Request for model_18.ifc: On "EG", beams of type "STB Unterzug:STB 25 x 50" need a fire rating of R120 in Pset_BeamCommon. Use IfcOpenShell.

First a look at what the model holds.

```python
import ifcopenshell
import ifcopenshell.util.element

model = ifcopenshell.open("model_18.ifc")
print(model.schema)
storey = next(s for s in model.by_type("IfcBuildingStorey") if s.Name == "EG")
beams = [e for e in ifcopenshell.util.element.get_decomposition(storey) if e.is_a("IfcBeam")]
seen = {}
for e in beams:
    element_type = ifcopenshell.util.element.get_type(e)
    key = (element_type.Name if element_type != e and element_type else None, ifcopenshell.util.element.get_pset(e, "Pset_BeamCommon", "FireRating"))
    seen[key] = seen.get(key, 0) + 1
for (name, value), count in sorted(seen.items(), key=str):
    print(count, "x", name, "|", value)
```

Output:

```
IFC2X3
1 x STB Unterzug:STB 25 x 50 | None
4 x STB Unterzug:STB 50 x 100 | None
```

```python
import ifcopenshell
import ifcopenshell.api.pset
import ifcopenshell.util.element

model = ifcopenshell.open("model_18.ifc")

storey = next(s for s in model.by_type("IfcBuildingStorey") if s.Name == "EG")
beams = [e for e in ifcopenshell.util.element.get_decomposition(storey) if e.is_a("IfcBeam")]

count = 0
for e in beams:
    element_type = ifcopenshell.util.element.get_type(e)
    if element_type in (None, e) or element_type.Name != "STB Unterzug:STB 25 x 50":
        continue
    # add_pset returns the element's existing set when there is one.
    pset = ifcopenshell.api.pset.add_pset(model, product=e, name="Pset_BeamCommon")
    ifcopenshell.api.pset.edit_pset(model, pset=pset, properties={"FireRating": "R120"})
    count += 1

print(count, "beams updated")

model.write("model_18_rev.ifc")
```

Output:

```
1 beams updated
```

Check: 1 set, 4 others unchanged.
